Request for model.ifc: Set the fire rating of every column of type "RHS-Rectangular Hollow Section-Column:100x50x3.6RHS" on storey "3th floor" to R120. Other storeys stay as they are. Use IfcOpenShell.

First a look at what the model holds.

```python
import ifcopenshell
import ifcopenshell.util.element

model = ifcopenshell.open("model.ifc")
print(model.schema)
storey = next(s for s in model.by_type("IfcBuildingStorey") if s.Name == "3th floor")
columns = [e for e in ifcopenshell.util.element.get_decomposition(storey) if e.is_a("IfcColumn")]
seen = {}
for e in columns:
    element_type = ifcopenshell.util.element.get_type(e)
    key = (element_type.Name if element_type != e and element_type else None, ifcopenshell.util.element.get_pset(e, "Pset_ColumnCommon", "FireRating"))
    seen[key] = seen.get(key, 0) + 1
for (name, value), count in sorted(seen.items(), key=str):
    print(count, "x", name, "|", value)
```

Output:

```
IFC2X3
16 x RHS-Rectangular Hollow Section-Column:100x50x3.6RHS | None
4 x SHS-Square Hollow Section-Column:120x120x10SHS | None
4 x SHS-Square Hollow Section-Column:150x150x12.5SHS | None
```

```python
import ifcopenshell
import ifcopenshell.api.pset
import ifcopenshell.util.element

model = ifcopenshell.open("model.ifc")

storey = next(s for s in model.by_type("IfcBuildingStorey") if s.Name == "3th floor")
columns = [e for e in ifcopenshell.util.element.get_decomposition(storey) if e.is_a("IfcColumn")]

count = 0
for e in columns:
    element_type = ifcopenshell.util.element.get_type(e)
    if element_type in (None, e) or element_type.Name != "RHS-Rectangular Hollow Section-Column:100x50x3.6RHS":
        continue
    # add_pset returns the element's existing set when there is one.
    pset = ifcopenshell.api.pset.add_pset(model, product=e, name="Pset_ColumnCommon")
    ifcopenshell.api.pset.edit_pset(model, pset=pset, properties={"FireRating": "R120"})
    count += 1

print(count, "columns updated")

model.write("model_edited.ifc")
```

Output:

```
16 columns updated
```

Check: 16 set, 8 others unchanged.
